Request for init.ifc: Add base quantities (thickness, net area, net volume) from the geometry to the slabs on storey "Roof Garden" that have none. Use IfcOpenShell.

First a look at what the model holds.

```python
import ifcopenshell
import ifcopenshell.util.element
import ifcopenshell.util.unit

model = ifcopenshell.open("init.ifc")
print(model.schema)
for unit_type in ("LENGTHUNIT", "AREAUNIT", "VOLUMEUNIT"):
    print(unit_type, ifcopenshell.util.unit.calculate_unit_scale(model, unit_type))
storey = next(s for s in model.by_type("IfcBuildingStorey") if s.Name == "Roof Garden")
slabs = [e for e in ifcopenshell.util.element.get_decomposition(storey) if e.is_a("IfcSlab")]
for e in sorted(slabs, key=lambda e: e.id()):
    print(e.id(), e.is_a(), e.Name, list(ifcopenshell.util.element.get_psets(e, qtos_only=True)), sep=" | ")
```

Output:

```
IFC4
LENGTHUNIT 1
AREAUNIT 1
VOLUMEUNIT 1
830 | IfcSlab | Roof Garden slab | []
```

```python
import ifcopenshell
import ifcopenshell.api.pset
import ifcopenshell.geom
import ifcopenshell.util.element
import ifcopenshell.util.shape
import ifcopenshell.util.unit

model = ifcopenshell.open("init.ifc")
unit_scale = ifcopenshell.util.unit.calculate_unit_scale(model)
area_scale = ifcopenshell.util.unit.calculate_unit_scale(model, "AREAUNIT")
volume_scale = ifcopenshell.util.unit.calculate_unit_scale(model, "VOLUMEUNIT")
settings = ifcopenshell.geom.settings()

storey = next(s for s in model.by_type("IfcBuildingStorey") if s.Name == "Roof Garden")
slabs = [e for e in ifcopenshell.util.element.get_decomposition(storey) if e.is_a("IfcSlab")]

for e in sorted(slabs, key=lambda e: e.id()):
    if ifcopenshell.util.element.get_psets(e, qtos_only=True, should_inherit=False):
        continue
    # Geometry comes back in metres, in the element's own axes.
    shape = ifcopenshell.geom.create_shape(settings, e)
    values = {
        "Width": ifcopenshell.util.shape.get_z(shape.geometry) / unit_scale,
        "NetArea": ifcopenshell.util.shape.get_footprint_area(shape.geometry) / area_scale,
        "NetVolume": ifcopenshell.util.shape.get_volume(shape.geometry) / volume_scale,
    }
    qto = ifcopenshell.api.pset.add_qto(model, product=e, name="Qto_SlabBaseQuantities")
    ifcopenshell.api.pset.edit_qto(model, qto=qto, properties=values)
    print(e.id(), {k: round(v, 3) for k, v in values.items()})

model.write("init_v2.ifc")
```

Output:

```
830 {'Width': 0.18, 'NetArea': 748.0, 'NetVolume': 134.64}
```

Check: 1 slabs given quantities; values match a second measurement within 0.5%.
